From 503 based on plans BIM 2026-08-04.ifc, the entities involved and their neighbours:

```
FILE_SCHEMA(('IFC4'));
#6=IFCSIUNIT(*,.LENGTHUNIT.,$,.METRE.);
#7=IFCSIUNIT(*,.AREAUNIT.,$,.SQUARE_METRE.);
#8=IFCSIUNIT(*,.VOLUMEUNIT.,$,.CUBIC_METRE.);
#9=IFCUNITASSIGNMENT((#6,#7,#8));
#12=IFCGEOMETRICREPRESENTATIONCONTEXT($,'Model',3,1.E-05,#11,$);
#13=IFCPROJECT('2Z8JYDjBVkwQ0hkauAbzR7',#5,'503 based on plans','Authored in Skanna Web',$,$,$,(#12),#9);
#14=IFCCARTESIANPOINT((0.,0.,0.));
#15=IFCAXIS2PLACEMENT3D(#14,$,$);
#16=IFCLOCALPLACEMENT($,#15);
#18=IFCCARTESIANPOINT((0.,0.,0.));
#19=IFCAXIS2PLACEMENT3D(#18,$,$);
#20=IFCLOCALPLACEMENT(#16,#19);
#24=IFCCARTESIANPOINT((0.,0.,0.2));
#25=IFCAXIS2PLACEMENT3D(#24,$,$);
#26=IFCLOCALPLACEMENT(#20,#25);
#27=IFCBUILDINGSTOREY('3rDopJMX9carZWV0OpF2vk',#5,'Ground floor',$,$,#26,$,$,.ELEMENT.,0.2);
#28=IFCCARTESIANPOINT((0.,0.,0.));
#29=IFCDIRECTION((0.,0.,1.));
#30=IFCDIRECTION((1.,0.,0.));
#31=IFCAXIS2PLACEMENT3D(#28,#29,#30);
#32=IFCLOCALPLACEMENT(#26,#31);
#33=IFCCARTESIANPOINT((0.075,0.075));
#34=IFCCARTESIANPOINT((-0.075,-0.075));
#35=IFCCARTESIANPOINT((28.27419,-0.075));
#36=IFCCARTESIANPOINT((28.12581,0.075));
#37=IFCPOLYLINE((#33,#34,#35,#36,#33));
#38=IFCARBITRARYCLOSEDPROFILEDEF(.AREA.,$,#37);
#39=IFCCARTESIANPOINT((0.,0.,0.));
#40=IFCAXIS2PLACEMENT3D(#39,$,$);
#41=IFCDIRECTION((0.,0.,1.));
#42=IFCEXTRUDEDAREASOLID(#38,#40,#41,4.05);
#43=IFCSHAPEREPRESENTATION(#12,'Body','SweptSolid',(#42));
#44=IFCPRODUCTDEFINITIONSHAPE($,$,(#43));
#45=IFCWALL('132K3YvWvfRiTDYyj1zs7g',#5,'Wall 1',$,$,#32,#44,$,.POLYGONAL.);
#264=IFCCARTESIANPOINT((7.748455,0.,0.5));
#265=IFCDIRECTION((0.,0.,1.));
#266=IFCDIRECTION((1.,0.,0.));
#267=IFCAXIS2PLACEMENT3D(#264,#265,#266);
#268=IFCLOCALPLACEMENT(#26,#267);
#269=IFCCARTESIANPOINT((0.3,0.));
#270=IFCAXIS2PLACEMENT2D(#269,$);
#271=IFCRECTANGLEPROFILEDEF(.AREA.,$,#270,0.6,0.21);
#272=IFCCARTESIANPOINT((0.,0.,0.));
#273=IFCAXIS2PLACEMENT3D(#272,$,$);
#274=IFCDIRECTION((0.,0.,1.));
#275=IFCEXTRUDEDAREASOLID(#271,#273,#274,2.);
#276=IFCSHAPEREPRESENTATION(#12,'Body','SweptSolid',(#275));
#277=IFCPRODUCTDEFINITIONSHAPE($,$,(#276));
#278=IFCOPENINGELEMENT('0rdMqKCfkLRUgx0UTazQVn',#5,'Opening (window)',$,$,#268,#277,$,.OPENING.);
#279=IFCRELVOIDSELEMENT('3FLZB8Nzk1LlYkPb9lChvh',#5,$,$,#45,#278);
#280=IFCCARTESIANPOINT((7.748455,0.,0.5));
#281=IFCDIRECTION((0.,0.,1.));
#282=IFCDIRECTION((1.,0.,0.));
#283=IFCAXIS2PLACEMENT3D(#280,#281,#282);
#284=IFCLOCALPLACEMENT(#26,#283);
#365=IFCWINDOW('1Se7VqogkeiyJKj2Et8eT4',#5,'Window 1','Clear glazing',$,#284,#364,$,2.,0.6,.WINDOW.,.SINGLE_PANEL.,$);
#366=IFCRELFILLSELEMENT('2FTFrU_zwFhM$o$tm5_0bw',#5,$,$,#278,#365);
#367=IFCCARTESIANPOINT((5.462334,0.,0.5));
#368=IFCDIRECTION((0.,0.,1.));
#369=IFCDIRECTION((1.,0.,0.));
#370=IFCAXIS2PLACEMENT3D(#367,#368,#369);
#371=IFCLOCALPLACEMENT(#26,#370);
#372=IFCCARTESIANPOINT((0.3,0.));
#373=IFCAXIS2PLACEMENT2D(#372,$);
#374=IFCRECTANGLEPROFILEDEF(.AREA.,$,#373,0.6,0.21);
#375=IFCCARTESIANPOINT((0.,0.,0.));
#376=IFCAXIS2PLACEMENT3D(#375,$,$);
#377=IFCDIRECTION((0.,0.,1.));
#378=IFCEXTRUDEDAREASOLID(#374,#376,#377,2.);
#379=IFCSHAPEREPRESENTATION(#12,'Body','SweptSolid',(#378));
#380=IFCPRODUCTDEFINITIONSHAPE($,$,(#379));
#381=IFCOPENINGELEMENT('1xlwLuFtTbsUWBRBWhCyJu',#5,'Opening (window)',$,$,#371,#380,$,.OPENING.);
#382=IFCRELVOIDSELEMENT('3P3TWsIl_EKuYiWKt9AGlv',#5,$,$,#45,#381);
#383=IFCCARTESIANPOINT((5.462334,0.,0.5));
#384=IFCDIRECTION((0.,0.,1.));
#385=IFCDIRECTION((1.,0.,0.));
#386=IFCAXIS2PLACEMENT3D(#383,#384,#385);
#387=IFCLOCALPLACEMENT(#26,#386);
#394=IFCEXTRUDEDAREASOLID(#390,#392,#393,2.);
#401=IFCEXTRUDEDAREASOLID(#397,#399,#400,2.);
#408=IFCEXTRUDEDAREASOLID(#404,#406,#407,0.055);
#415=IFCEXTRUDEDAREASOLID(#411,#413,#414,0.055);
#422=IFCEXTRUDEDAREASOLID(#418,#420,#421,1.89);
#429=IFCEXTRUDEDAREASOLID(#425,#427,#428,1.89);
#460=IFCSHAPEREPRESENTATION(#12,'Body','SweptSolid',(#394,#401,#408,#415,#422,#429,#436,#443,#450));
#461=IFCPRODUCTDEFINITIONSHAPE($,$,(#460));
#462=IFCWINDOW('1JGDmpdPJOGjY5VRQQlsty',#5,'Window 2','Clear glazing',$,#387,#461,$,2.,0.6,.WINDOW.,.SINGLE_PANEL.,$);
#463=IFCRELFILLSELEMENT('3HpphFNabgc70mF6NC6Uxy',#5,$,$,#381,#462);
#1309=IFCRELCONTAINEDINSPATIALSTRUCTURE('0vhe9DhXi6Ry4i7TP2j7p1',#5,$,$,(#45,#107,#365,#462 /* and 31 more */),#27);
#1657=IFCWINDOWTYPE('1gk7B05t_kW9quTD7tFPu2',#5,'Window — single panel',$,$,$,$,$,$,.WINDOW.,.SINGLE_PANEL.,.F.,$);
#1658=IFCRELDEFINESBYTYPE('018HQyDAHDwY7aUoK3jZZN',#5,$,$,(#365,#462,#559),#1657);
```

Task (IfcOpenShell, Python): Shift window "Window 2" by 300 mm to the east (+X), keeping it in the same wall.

```python
import ifcopenshell
import ifcopenshell.api.geometry
import ifcopenshell.util.placement
import ifcopenshell.util.unit

model = ifcopenshell.open("503 based on plans BIM 2026-08-04.ifc")
unit_scale = ifcopenshell.util.unit.calculate_unit_scale(model)

window = model.by_guid("1JGDmpdPJOGjY5VRQQlsty")
opening = window.FillsVoids[0].RelatingOpeningElement
wall = opening.VoidsElements[0].RelatingBuildingElement

wall_matrix = ifcopenshell.util.placement.get_local_placement(wall.ObjectPlacement)
shift = wall_matrix[:3, 0] * 0.3 / unit_scale
before = ifcopenshell.util.placement.get_local_placement(window.ObjectPlacement)[:3, 3].copy()

# The window is not placed relative to its opening, so move both.
for product in (opening, window):
    matrix = ifcopenshell.util.placement.get_local_placement(product.ObjectPlacement)
    matrix[:3, 3] += shift
    ifcopenshell.api.geometry.edit_object_placement(model, product=product, matrix=matrix, is_si=False)

after = ifcopenshell.util.placement.get_local_placement(window.ObjectPlacement)[:3, 3]
print("window moved by", (after - before).round(3) + 0.0)

model.write("503 based on plans BIM 2026-08-04_rev.ifc")
```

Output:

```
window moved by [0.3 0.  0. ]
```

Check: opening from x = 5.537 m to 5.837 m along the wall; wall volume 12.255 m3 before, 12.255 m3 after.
